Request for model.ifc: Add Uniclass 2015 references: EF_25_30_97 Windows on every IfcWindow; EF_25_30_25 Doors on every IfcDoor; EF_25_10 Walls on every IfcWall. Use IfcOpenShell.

First a look at what the model holds.

```python
import ifcopenshell

model = ifcopenshell.open("model.ifc")
print(model.schema)
print("classifications:", [c.Name for c in model.by_type("IfcClassification")])
for ifc_class in ("IfcDoor", "IfcRoof", "IfcStair", "IfcWall", "IfcWindow"):
    print(ifc_class, len(model.by_type(ifc_class)))
```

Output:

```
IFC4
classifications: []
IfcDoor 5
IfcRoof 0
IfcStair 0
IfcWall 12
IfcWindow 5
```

```python
import ifcopenshell
import ifcopenshell.api.classification

model = ifcopenshell.open("model.ifc")

system = ifcopenshell.api.classification.add_classification(model, classification="Uniclass 2015")

codes = {
    "IfcWindow": ("EF_25_30_97", "Windows"),
    "IfcDoor": ("EF_25_30_25", "Doors"),
    "IfcWall": ("EF_25_10", "Walls"),
}
for ifc_class, (code, name) in codes.items():
    products = model.by_type(ifc_class)
    ifcopenshell.api.classification.add_reference(
        model, products=products, classification=system, identification=code, name=name
    )
    print(code, len(products))

model.write("model-out.ifc")
```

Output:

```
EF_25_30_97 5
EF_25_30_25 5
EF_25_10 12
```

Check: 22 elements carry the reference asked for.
